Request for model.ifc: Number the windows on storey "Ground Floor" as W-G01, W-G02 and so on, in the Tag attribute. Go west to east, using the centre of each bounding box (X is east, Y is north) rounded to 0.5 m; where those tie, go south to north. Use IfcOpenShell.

First a look at what the model holds.

```python
import ifcopenshell
import ifcopenshell.util.element
import ifcopenshell.util.placement

model = ifcopenshell.open("model.ifc")
print(model.schema)
storey = next(s for s in model.by_type("IfcBuildingStorey") if s.Name == "Ground Floor")
windows = [e for e in ifcopenshell.util.element.get_decomposition(storey) if e.is_a("IfcWindow")]
for e in sorted(windows, key=lambda e: e.id()):
    origin = ifcopenshell.util.placement.get_local_placement(e.ObjectPlacement)[:3, 3]
    print(e.id(), e.Tag, e.Name, origin.round(2) + 0.0, sep=" | ")
```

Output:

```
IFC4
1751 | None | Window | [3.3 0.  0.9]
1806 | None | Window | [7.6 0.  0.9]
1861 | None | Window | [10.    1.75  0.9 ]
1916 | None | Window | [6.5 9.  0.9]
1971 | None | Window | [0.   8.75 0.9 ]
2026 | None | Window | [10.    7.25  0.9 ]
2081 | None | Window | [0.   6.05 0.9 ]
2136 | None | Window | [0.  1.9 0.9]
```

```python
import ifcopenshell
import ifcopenshell.geom
import ifcopenshell.util.element
import ifcopenshell.util.shape

model = ifcopenshell.open("model.ifc")
settings = ifcopenshell.geom.settings()
settings.set("use-world-coords", True)


def centre(element):
    shape = ifcopenshell.geom.create_shape(settings, element)
    return ifcopenshell.util.shape.get_bbox_centroid(shape.geometry)


storey = next(s for s in model.by_type("IfcBuildingStorey") if s.Name == "Ground Floor")
windows = [e for e in ifcopenshell.util.element.get_decomposition(storey) if e.is_a("IfcWindow")]

# Insertion points can sit at a corner or the storey origin, so sort by the geometry (in metres).
centres = {e: centre(e) for e in windows}
windows.sort(key=lambda e: (round(centres[e][0] / 0.5), centres[e][1]))

for i, e in enumerate(windows, start=1):
    number = f"W-G{i:02d}"
    e.Tag = number
    print(e.id(), number)

model.write("model_rev.ifc")
```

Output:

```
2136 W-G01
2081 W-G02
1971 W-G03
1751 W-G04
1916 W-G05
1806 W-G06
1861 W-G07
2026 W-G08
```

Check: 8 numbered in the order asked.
